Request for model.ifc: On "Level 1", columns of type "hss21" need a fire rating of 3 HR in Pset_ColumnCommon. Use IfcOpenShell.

First a look at what the model holds.

```python
import ifcopenshell
import ifcopenshell.util.element

model = ifcopenshell.open("model.ifc")
print(model.schema)
storey = next(s for s in model.by_type("IfcBuildingStorey") if s.Name == "Level 1")
columns = [e for e in ifcopenshell.util.element.get_decomposition(storey) if e.is_a("IfcColumn")]
seen = {}
for e in columns:
    element_type = ifcopenshell.util.element.get_type(e)
    key = (element_type.Name if element_type != e and element_type else None, ifcopenshell.util.element.get_pset(e, "Pset_ColumnCommon", "FireRating"))
    seen[key] = seen.get(key, 0) + 1
for (name, value), count in sorted(seen.items(), key=str):
    print(count, "x", name, "|", value)
```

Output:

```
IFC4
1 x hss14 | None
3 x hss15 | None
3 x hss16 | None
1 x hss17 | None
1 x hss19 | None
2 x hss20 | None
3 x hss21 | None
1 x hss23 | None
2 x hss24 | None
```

```python
import ifcopenshell
import ifcopenshell.api.pset
import ifcopenshell.util.element

model = ifcopenshell.open("model.ifc")

storey = next(s for s in model.by_type("IfcBuildingStorey") if s.Name == "Level 1")
columns = [e for e in ifcopenshell.util.element.get_decomposition(storey) if e.is_a("IfcColumn")]

count = 0
for e in columns:
    element_type = ifcopenshell.util.element.get_type(e)
    if element_type in (None, e) or element_type.Name != "hss21":
        continue
    # add_pset returns the element's existing set when there is one.
    pset = ifcopenshell.api.pset.add_pset(model, product=e, name="Pset_ColumnCommon")
    ifcopenshell.api.pset.edit_pset(model, pset=pset, properties={"FireRating": "3 HR"})
    count += 1

print(count, "columns updated")

model.write("model_v2.ifc")
```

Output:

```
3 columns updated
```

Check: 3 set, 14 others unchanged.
